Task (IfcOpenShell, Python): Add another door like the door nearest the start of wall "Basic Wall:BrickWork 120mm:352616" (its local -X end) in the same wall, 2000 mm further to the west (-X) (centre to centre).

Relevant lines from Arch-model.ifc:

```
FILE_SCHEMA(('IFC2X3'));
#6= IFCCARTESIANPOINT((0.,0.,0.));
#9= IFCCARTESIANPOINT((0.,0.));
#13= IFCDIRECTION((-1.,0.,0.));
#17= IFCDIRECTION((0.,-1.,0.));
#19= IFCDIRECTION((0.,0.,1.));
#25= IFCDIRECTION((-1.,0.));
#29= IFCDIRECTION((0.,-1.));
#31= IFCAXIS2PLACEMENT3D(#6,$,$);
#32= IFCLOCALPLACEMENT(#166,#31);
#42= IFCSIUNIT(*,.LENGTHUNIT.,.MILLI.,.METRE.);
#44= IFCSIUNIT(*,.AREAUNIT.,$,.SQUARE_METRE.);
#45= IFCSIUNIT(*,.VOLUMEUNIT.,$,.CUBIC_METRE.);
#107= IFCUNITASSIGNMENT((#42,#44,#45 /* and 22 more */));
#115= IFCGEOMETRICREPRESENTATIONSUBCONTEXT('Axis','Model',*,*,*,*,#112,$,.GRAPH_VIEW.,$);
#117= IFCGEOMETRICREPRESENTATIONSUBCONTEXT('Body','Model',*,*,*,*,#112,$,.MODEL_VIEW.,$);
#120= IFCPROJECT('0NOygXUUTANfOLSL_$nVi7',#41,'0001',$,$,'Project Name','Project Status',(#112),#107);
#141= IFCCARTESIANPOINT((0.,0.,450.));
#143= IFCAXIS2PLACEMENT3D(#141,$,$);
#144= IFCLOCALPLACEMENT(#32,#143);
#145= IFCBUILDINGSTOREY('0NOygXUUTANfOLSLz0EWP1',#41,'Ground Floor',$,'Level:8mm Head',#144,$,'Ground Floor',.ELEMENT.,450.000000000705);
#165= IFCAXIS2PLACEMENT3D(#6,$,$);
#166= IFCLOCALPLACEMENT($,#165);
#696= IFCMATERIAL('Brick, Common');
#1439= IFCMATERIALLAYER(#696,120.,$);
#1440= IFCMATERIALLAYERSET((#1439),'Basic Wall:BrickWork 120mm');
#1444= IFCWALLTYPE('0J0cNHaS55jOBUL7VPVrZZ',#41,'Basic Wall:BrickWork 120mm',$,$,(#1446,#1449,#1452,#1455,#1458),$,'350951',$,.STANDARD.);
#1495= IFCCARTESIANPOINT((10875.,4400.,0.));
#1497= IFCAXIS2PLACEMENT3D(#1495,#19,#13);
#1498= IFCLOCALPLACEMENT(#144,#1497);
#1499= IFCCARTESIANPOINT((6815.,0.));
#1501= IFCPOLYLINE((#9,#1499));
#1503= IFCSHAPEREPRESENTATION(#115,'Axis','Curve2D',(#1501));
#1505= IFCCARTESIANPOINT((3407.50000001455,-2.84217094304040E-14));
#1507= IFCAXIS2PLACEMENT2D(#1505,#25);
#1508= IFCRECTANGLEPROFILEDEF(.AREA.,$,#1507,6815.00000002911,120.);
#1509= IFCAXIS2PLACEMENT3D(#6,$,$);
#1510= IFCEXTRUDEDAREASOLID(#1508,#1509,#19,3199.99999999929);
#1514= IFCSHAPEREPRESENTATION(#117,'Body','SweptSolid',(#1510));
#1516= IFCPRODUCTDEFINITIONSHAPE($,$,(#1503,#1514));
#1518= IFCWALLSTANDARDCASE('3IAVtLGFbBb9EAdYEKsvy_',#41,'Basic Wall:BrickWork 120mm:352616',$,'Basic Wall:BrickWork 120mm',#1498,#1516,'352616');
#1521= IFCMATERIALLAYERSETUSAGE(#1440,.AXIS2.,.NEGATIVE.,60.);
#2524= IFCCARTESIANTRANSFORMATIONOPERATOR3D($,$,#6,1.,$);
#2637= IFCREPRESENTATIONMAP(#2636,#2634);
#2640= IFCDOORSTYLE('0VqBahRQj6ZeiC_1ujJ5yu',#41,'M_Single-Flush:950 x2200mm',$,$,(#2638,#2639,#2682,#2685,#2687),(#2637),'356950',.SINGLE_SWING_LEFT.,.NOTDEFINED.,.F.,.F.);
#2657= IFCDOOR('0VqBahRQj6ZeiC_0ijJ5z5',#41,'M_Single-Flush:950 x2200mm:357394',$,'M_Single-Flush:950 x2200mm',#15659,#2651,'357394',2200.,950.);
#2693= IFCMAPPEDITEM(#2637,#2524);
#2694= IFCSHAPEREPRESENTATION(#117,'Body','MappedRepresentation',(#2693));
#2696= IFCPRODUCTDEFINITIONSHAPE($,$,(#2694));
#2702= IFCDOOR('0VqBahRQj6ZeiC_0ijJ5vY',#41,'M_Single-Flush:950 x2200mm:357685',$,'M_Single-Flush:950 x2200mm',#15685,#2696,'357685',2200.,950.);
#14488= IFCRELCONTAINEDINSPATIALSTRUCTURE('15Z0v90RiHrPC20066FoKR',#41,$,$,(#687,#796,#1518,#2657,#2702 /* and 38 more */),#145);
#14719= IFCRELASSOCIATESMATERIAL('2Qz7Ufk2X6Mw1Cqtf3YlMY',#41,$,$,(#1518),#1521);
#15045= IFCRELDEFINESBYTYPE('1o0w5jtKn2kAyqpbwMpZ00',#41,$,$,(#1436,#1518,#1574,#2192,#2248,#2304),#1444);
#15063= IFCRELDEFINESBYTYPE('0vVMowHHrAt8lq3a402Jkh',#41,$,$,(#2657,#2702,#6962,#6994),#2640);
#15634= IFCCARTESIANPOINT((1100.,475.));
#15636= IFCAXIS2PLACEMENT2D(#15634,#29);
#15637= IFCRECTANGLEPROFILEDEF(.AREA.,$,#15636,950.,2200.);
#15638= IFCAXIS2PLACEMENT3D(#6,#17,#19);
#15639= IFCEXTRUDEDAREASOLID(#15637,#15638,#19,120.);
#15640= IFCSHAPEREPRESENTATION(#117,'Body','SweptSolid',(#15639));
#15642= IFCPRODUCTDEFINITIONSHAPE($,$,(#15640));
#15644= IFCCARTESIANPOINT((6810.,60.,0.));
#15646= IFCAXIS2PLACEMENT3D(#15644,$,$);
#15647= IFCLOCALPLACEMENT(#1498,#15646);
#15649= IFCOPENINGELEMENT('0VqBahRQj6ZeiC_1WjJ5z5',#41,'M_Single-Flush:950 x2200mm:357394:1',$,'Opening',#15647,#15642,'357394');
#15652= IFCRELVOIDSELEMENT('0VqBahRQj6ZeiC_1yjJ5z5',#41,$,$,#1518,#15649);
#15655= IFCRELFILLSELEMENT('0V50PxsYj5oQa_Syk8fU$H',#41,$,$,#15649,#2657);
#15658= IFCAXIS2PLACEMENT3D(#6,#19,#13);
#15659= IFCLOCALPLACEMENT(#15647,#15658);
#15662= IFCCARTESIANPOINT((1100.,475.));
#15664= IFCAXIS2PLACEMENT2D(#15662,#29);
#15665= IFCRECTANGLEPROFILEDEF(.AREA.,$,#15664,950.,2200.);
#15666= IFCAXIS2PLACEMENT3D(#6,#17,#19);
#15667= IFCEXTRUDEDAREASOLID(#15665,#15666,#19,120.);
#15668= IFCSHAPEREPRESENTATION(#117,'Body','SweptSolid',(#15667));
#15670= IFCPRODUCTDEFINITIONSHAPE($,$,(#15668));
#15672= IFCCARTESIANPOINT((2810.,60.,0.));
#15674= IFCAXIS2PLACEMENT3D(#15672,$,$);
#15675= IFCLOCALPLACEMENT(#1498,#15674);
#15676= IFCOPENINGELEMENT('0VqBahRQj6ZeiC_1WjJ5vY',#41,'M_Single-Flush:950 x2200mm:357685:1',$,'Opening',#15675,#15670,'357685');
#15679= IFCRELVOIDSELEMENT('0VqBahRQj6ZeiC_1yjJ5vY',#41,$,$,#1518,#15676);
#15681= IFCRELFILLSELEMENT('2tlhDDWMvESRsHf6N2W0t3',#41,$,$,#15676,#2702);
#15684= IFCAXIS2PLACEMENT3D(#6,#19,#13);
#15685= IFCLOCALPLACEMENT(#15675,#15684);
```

```python
import ifcopenshell
import ifcopenshell.api.feature
import ifcopenshell.api.geometry
import ifcopenshell.api.root
import ifcopenshell.geom
import ifcopenshell.util.element
import ifcopenshell.util.placement
import ifcopenshell.util.shape
import ifcopenshell.util.unit

model = ifcopenshell.open("Arch-model.ifc")
unit_scale = ifcopenshell.util.unit.calculate_unit_scale(model)
settings = ifcopenshell.geom.settings()


def volume(element):
    """Net volume in cubic metres, openings subtracted."""
    shape = ifcopenshell.geom.create_shape(settings, element)
    return ifcopenshell.util.shape.get_volume(shape.geometry)


def reuse_history(source, copy):
    """copy_class also copies each property set's owner history, people and application; keep the originals."""
    for rel in copy.IsDefinedBy:
        if rel.is_a("IfcRelDefinesByProperties") and (history := rel.RelatingPropertyDefinition.OwnerHistory):
            rel.RelatingPropertyDefinition.OwnerHistory = source.OwnerHistory
            ifcopenshell.util.element.remove_deep2(model, history)


door = model.by_id(2702)
opening = door.FillsVoids[0].RelatingOpeningElement
wall = opening.VoidsElements[0].RelatingBuildingElement
before = volume(wall)
shift = ifcopenshell.util.placement.get_local_placement(wall.ObjectPlacement)[:3, 0] * 2 / unit_scale

# copy_class copies the void relationship, type, container and properties, but no geometry.
new_opening = ifcopenshell.api.root.copy_class(model, product=opening)
new_opening.Representation = ifcopenshell.util.element.copy_deep(
    model, opening.Representation, exclude=["IfcGeometricRepresentationContext", "IfcRepresentationMap"]
)
new_opening.Name = "M_Single-Flush:950 x2200mm"
new_opening.Tag = None
new_door = ifcopenshell.api.root.copy_class(model, product=door)
new_door.Representation = ifcopenshell.util.element.copy_deep(
    model, door.Representation, exclude=["IfcGeometricRepresentationContext", "IfcRepresentationMap"]
)
new_door.Name = "M_Single-Flush:950 x2200mm"
new_door.Tag = None
reuse_history(door, new_door)
fills = ifcopenshell.api.feature.add_filling(model, opening=new_opening, element=new_door)
fills.OwnerHistory = new_door.OwnerHistory  # required in IFC2X3

for old, new in ((opening, new_opening), (door, new_door)):
    matrix = ifcopenshell.util.placement.get_local_placement(old.ObjectPlacement)
    matrix[:3, 3] += shift
    ifcopenshell.api.geometry.edit_object_placement(model, product=new, matrix=matrix, is_si=False)

after = volume(wall)

print(f"wall volume {before:.3f} -> {after:.3f} m3")

model.write("Arch-model_updated.ifc")
```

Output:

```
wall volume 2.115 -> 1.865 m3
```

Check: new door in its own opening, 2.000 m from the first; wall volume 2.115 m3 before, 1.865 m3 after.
